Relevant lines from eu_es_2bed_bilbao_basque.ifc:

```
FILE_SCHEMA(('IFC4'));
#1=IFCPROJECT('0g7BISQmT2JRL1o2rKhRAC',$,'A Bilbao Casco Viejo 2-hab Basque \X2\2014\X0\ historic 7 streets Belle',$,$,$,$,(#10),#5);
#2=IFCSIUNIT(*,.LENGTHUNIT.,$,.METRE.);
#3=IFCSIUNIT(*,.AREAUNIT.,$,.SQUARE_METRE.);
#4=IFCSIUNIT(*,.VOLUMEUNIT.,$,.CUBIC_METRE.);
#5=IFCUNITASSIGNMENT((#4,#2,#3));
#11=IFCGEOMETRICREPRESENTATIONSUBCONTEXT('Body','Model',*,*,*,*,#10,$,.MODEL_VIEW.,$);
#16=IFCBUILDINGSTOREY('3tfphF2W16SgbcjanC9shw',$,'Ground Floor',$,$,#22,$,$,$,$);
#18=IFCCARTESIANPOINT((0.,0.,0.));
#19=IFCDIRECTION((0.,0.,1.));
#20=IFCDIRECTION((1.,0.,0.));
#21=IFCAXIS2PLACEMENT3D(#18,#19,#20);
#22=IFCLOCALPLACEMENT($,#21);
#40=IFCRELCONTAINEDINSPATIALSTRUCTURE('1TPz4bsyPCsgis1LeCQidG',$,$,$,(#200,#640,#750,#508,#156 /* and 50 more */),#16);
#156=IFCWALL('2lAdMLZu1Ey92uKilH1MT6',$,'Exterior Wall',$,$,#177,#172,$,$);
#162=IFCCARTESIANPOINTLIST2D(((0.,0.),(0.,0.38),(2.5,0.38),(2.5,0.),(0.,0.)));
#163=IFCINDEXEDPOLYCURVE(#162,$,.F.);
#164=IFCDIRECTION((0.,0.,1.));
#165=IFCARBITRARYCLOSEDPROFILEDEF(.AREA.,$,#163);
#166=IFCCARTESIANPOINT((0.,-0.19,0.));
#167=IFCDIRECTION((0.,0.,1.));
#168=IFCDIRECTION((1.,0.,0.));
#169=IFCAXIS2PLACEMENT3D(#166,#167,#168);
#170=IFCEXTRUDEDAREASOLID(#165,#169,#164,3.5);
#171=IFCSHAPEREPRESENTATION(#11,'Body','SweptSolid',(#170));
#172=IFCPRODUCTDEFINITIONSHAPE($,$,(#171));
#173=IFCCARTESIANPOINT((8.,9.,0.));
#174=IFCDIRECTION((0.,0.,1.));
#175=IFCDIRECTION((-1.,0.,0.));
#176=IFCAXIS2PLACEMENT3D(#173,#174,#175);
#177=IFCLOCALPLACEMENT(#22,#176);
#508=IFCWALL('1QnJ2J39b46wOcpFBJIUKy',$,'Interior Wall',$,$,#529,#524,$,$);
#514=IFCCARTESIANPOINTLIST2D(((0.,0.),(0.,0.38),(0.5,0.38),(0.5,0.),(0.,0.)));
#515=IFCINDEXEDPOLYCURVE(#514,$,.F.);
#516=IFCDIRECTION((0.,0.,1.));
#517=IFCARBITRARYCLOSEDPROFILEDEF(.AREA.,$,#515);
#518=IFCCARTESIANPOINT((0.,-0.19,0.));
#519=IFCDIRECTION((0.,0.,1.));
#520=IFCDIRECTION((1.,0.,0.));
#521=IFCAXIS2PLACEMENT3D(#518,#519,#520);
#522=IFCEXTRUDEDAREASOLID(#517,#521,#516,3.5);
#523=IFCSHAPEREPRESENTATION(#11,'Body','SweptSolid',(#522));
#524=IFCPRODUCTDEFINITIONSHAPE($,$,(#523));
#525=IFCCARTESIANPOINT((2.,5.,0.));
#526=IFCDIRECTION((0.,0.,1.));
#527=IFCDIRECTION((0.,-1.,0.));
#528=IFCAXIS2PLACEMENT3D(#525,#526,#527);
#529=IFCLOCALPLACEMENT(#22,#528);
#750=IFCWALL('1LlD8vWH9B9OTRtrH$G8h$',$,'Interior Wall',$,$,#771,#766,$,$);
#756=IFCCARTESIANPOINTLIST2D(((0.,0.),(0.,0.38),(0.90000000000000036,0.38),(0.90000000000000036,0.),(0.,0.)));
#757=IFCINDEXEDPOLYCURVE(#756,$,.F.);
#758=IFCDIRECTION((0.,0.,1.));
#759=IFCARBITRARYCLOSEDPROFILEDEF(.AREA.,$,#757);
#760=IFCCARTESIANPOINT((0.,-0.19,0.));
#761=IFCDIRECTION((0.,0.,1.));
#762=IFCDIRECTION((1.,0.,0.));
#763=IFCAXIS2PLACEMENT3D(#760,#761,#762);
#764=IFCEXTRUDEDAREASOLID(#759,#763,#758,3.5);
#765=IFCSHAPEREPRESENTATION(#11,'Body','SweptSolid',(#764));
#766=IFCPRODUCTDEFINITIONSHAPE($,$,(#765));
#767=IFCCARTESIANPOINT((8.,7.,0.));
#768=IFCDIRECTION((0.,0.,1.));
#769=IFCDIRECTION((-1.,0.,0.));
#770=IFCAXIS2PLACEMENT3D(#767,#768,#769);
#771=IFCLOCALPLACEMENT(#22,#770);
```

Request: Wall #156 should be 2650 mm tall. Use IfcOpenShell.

```python
import ifcopenshell
import ifcopenshell.geom
import ifcopenshell.util.representation
import ifcopenshell.util.shape

model = ifcopenshell.open("eu_es_2bed_bilbao_basque.ifc")
settings = ifcopenshell.geom.settings()


def volume(element):
    """Net volume in cubic metres, openings subtracted."""
    shape = ifcopenshell.geom.create_shape(settings, element)
    return ifcopenshell.util.shape.get_volume(shape.geometry)


wall = model.by_guid("2lAdMLZu1Ey92uKilH1MT6")
before = volume(wall)

body = ifcopenshell.util.representation.get_representation(wall, "Model", "Body")
solid = body.Items[0]
old_height = solid.Depth
solid.Depth = 2.65
after = volume(wall)

print(f"height {old_height:g} -> {solid.Depth:g}, volume {before:.3f} -> {after:.3f} m3")

model.write("eu_es_2bed_bilbao_basque_updated.ifc")
```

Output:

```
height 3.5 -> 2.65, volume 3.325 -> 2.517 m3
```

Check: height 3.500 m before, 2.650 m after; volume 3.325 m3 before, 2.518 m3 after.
